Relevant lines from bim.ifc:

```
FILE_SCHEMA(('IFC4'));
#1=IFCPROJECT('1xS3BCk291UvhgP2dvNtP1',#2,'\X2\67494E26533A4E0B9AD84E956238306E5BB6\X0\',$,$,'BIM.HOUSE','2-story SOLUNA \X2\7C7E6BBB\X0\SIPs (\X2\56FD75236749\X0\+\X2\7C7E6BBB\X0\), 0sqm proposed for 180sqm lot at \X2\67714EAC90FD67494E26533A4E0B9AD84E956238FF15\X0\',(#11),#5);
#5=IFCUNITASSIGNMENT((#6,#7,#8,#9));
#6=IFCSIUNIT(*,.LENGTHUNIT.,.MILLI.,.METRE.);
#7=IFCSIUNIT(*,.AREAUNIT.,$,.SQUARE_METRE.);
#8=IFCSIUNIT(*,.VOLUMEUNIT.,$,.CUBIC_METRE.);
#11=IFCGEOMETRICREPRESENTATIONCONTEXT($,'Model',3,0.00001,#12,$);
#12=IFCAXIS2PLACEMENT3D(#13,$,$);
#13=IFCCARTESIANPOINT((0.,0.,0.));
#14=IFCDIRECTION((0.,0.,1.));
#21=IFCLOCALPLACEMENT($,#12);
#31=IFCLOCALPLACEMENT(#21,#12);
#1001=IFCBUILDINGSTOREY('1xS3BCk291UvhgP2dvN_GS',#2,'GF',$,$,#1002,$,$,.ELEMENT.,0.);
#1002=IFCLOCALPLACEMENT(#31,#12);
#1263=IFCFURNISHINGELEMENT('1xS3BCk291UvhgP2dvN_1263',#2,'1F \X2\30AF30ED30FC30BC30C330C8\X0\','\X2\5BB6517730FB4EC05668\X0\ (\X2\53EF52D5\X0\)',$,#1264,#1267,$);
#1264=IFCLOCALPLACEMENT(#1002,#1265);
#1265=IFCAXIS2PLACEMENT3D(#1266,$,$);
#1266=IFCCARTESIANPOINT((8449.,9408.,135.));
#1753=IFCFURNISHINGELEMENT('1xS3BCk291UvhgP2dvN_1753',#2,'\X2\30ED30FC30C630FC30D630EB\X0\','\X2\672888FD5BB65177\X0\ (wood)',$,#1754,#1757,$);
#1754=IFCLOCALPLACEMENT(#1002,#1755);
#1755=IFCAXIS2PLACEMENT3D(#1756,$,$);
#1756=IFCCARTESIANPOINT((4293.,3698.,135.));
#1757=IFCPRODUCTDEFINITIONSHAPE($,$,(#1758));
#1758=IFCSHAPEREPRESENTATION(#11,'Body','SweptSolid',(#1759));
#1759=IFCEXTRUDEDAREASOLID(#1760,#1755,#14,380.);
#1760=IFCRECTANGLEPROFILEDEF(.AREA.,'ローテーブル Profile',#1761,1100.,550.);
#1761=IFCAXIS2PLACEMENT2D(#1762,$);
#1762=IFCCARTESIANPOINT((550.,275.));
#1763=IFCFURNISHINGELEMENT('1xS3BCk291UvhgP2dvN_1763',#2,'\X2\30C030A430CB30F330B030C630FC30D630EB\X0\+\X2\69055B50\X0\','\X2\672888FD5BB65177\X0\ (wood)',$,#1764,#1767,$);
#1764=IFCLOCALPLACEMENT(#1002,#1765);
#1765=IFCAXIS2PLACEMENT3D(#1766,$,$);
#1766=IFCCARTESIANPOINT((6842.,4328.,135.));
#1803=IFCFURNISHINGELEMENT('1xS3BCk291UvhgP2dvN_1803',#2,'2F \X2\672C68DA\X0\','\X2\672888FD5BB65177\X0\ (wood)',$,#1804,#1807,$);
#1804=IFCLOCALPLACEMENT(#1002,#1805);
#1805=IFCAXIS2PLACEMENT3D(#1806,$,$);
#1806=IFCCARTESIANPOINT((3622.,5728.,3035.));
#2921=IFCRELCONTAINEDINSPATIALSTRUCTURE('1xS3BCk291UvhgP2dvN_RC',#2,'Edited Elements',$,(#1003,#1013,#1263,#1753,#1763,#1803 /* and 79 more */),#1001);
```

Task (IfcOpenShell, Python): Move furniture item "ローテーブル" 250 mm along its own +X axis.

```python
import ifcopenshell
import ifcopenshell.api.geometry
import ifcopenshell.util.placement
import ifcopenshell.util.unit

model = ifcopenshell.open("bim.ifc")
unit_scale = ifcopenshell.util.unit.calculate_unit_scale(model)

item = model.by_guid("1xS3BCk291UvhgP2dvN_1753")
matrix = ifcopenshell.util.placement.get_local_placement(item.ObjectPlacement)
matrix[:3, 3] += matrix[:3, 0] * 0.25 / unit_scale
ifcopenshell.api.geometry.edit_object_placement(model, product=item, matrix=matrix, is_si=False)

print(ifcopenshell.util.placement.get_local_placement(item.ObjectPlacement).round(3) + 0.0)

model.write("bim-out.ifc")
```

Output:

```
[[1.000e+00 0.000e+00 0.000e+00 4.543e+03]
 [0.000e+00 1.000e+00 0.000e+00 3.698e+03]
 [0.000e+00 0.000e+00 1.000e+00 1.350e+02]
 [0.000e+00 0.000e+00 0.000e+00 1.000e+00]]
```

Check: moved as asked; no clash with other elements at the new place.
